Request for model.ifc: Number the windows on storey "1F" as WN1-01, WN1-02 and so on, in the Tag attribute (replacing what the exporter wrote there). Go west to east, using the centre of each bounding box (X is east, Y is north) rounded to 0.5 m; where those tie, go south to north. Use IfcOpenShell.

First a look at what the model holds.

```python
import ifcopenshell
import ifcopenshell.util.element
import ifcopenshell.util.placement

model = ifcopenshell.open("model.ifc")
print(model.schema)
storey = next(s for s in model.by_type("IfcBuildingStorey") if s.Name == "1F")
windows = [e for e in ifcopenshell.util.element.get_decomposition(storey) if e.is_a("IfcWindow")]
for e in sorted(windows, key=lambda e: e.id()):
    origin = ifcopenshell.util.placement.get_local_placement(e.ObjectPlacement)[:3, 3]
    print(e.id(), e.Tag, e.Name, origin.round(2) + 0.0, sep=" | ")
```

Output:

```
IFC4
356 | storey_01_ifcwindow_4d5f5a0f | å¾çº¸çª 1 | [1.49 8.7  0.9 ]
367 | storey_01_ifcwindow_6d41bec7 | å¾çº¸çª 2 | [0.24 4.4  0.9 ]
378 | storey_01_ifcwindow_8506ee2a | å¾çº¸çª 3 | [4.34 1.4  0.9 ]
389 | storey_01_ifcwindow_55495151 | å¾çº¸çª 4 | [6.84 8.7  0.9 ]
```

```python
import ifcopenshell
import ifcopenshell.geom
import ifcopenshell.util.element
import ifcopenshell.util.shape

model = ifcopenshell.open("model.ifc")
settings = ifcopenshell.geom.settings()
settings.set("use-world-coords", True)


def centre(element):
    shape = ifcopenshell.geom.create_shape(settings, element)
    return ifcopenshell.util.shape.get_bbox_centroid(shape.geometry)


storey = next(s for s in model.by_type("IfcBuildingStorey") if s.Name == "1F")
windows = [e for e in ifcopenshell.util.element.get_decomposition(storey) if e.is_a("IfcWindow")]

# Insertion points can sit at a corner or the storey origin, so sort by the geometry (in metres).
centres = {e: centre(e) for e in windows}
windows.sort(key=lambda e: (round(centres[e][0] / 0.5), centres[e][1]))

for i, e in enumerate(windows, start=1):
    number = f"WN1-{i:02d}"
    e.Tag = number
    print(e.id(), number)

model.write("model_edited.ifc")
```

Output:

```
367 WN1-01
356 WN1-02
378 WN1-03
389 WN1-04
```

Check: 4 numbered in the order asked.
